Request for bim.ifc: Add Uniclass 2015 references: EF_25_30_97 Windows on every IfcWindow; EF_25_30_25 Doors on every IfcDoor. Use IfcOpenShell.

First a look at what the model holds.

```python
import ifcopenshell

model = ifcopenshell.open("bim.ifc")
print(model.schema)
print("classifications:", [c.Name for c in model.by_type("IfcClassification")])
for ifc_class in ("IfcDoor", "IfcRoof", "IfcStair", "IfcWall", "IfcWindow"):
    print(ifc_class, len(model.by_type(ifc_class)))
```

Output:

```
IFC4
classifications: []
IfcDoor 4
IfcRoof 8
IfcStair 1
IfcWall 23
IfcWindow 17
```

```python
import ifcopenshell
import ifcopenshell.api.classification

model = ifcopenshell.open("bim.ifc")

system = ifcopenshell.api.classification.add_classification(model, classification="Uniclass 2015")

codes = {
    "IfcWindow": ("EF_25_30_97", "Windows"),
    "IfcDoor": ("EF_25_30_25", "Doors"),
}
for ifc_class, (code, name) in codes.items():
    products = model.by_type(ifc_class)
    ifcopenshell.api.classification.add_reference(
        model, products=products, classification=system, identification=code, name=name
    )
    print(code, len(products))

model.write("bim-out.ifc")
```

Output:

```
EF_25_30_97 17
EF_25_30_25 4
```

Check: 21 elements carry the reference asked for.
